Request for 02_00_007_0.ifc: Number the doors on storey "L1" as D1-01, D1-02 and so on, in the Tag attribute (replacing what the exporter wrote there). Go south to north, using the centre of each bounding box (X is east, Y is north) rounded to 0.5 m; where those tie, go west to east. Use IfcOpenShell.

First a look at what the model holds.

```python
import ifcopenshell
import ifcopenshell.util.element
import ifcopenshell.util.placement

model = ifcopenshell.open("02_00_007_0.ifc")
print(model.schema)
storey = next(s for s in model.by_type("IfcBuildingStorey") if s.Name == "L1")
doors = [e for e in ifcopenshell.util.element.get_decomposition(storey) if e.is_a("IfcDoor")]
for e in sorted(doors, key=lambda e: e.id()):
    origin = ifcopenshell.util.placement.get_local_placement(e.ObjectPlacement)[:3, 3]
    print(e.id(), e.Tag, e.Name, origin.round(2) + 0.0, sep=" | ")
```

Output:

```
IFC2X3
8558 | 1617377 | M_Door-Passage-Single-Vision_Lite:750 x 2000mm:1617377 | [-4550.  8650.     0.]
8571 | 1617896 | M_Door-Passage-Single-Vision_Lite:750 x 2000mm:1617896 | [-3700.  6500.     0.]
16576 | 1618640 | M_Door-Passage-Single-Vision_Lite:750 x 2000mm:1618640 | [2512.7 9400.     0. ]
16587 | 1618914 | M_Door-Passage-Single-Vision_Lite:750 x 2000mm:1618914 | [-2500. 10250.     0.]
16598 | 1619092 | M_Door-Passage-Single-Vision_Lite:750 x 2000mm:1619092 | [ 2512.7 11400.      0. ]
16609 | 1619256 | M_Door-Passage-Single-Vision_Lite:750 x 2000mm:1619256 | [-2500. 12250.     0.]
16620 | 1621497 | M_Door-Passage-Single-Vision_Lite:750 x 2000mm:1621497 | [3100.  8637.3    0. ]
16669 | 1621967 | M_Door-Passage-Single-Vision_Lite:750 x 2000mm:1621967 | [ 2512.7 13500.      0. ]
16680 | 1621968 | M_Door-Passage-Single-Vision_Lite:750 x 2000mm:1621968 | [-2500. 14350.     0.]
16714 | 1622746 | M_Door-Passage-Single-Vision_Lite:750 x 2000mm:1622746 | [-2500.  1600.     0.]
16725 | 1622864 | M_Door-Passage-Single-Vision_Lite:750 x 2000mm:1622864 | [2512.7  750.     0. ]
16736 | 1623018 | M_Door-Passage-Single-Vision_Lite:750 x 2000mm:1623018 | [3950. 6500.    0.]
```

```python
import ifcopenshell
import ifcopenshell.geom
import ifcopenshell.util.element
import ifcopenshell.util.shape

model = ifcopenshell.open("02_00_007_0.ifc")
settings = ifcopenshell.geom.settings()
settings.set("use-world-coords", True)


def centre(element):
    shape = ifcopenshell.geom.create_shape(settings, element)
    return ifcopenshell.util.shape.get_bbox_centroid(shape.geometry)


storey = next(s for s in model.by_type("IfcBuildingStorey") if s.Name == "L1")
doors = [e for e in ifcopenshell.util.element.get_decomposition(storey) if e.is_a("IfcDoor")]

# Insertion points can sit at a corner or the storey origin, so sort by the geometry (in metres).
centres = {e: centre(e) for e in doors}
doors.sort(key=lambda e: (round(centres[e][1] / 0.5), centres[e][0]))

for i, e in enumerate(doors, start=1):
    number = f"D1-{i:02d}"
    e.Tag = number
    print(e.id(), number)

model.write("02_00_007_0-out.ifc")
```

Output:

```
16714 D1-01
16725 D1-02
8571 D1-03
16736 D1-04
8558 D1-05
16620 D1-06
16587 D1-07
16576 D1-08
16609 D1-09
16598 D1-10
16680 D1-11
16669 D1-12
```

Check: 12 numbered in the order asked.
